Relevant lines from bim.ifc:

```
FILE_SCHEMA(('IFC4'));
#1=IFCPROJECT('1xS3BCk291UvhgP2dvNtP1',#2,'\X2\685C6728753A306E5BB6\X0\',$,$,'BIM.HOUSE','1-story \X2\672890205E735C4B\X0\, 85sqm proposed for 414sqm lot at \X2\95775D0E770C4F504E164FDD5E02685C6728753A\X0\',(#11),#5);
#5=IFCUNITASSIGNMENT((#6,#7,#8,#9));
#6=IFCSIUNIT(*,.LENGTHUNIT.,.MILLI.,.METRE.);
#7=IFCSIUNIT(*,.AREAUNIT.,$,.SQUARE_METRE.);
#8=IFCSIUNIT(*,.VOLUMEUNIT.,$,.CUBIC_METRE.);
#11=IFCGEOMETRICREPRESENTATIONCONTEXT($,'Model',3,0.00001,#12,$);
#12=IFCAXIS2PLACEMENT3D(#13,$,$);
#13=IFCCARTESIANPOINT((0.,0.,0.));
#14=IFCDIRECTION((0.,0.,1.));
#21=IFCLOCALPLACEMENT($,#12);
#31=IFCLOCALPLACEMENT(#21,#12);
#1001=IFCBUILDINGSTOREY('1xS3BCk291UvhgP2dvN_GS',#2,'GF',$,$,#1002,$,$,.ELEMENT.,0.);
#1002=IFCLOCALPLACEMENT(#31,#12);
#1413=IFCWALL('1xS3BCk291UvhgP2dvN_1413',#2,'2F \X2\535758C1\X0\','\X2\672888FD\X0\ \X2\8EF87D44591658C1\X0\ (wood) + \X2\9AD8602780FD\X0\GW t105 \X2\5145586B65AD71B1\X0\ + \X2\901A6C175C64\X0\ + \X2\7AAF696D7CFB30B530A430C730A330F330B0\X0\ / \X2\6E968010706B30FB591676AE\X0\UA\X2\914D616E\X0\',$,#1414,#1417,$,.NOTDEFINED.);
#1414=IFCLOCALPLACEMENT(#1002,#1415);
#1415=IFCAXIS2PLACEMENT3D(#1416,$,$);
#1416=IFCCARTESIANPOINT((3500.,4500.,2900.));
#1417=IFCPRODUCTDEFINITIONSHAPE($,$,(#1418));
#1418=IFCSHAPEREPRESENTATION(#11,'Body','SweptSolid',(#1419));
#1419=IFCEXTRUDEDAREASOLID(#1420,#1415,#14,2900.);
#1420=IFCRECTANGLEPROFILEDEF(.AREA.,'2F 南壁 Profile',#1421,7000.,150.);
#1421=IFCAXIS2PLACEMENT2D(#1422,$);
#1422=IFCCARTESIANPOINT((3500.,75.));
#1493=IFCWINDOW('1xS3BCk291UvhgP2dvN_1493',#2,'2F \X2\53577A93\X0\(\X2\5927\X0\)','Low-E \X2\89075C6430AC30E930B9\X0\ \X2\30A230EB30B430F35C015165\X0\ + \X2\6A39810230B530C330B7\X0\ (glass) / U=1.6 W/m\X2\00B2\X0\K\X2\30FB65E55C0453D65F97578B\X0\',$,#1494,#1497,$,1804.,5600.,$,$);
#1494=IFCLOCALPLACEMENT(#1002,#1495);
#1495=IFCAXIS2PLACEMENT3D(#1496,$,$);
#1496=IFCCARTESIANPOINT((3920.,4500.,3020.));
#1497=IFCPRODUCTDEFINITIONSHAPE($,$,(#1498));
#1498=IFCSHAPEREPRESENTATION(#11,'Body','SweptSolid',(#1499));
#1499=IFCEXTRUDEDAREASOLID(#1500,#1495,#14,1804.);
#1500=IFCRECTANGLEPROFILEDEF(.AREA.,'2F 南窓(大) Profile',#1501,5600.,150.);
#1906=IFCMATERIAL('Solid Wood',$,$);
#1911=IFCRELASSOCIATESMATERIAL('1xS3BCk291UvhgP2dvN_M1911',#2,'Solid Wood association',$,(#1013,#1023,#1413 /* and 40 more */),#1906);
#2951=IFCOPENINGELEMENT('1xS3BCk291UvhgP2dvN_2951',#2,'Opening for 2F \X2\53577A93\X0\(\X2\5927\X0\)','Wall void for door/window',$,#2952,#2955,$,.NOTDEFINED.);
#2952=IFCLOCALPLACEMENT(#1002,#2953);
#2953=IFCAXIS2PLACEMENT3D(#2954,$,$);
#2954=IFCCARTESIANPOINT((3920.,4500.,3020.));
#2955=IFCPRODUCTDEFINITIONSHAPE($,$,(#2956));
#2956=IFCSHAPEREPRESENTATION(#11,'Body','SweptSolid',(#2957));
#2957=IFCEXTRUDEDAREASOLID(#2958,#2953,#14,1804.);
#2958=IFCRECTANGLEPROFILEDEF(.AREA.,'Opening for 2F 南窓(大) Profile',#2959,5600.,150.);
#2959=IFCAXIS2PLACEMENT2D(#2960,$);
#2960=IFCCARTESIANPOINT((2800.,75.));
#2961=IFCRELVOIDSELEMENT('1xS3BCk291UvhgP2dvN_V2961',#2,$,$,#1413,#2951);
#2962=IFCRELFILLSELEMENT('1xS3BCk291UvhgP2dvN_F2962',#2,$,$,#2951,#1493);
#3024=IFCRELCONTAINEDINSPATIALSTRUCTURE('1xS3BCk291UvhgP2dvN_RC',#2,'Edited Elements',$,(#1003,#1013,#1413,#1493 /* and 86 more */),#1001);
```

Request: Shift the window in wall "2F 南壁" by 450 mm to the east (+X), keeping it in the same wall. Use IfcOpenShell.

```python
import ifcopenshell
import ifcopenshell.api.geometry
import ifcopenshell.util.placement
import ifcopenshell.util.unit

model = ifcopenshell.open("bim.ifc")
unit_scale = ifcopenshell.util.unit.calculate_unit_scale(model)

window = model.by_id(1493)
opening = window.FillsVoids[0].RelatingOpeningElement
wall = opening.VoidsElements[0].RelatingBuildingElement

wall_matrix = ifcopenshell.util.placement.get_local_placement(wall.ObjectPlacement)
shift = wall_matrix[:3, 0] * 0.45 / unit_scale
before = ifcopenshell.util.placement.get_local_placement(window.ObjectPlacement)[:3, 3].copy()

# The window is not placed relative to its opening, so move both.
for product in (opening, window):
    matrix = ifcopenshell.util.placement.get_local_placement(product.ObjectPlacement)
    matrix[:3, 3] += shift
    ifcopenshell.api.geometry.edit_object_placement(model, product=product, matrix=matrix, is_si=False)

after = ifcopenshell.util.placement.get_local_placement(window.ObjectPlacement)[:3, 3]
print("window moved by", (after - before).round(3) + 0.0)

model.write("bim_rev.ifc")
```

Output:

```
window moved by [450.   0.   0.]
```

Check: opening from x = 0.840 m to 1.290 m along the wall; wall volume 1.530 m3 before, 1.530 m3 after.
